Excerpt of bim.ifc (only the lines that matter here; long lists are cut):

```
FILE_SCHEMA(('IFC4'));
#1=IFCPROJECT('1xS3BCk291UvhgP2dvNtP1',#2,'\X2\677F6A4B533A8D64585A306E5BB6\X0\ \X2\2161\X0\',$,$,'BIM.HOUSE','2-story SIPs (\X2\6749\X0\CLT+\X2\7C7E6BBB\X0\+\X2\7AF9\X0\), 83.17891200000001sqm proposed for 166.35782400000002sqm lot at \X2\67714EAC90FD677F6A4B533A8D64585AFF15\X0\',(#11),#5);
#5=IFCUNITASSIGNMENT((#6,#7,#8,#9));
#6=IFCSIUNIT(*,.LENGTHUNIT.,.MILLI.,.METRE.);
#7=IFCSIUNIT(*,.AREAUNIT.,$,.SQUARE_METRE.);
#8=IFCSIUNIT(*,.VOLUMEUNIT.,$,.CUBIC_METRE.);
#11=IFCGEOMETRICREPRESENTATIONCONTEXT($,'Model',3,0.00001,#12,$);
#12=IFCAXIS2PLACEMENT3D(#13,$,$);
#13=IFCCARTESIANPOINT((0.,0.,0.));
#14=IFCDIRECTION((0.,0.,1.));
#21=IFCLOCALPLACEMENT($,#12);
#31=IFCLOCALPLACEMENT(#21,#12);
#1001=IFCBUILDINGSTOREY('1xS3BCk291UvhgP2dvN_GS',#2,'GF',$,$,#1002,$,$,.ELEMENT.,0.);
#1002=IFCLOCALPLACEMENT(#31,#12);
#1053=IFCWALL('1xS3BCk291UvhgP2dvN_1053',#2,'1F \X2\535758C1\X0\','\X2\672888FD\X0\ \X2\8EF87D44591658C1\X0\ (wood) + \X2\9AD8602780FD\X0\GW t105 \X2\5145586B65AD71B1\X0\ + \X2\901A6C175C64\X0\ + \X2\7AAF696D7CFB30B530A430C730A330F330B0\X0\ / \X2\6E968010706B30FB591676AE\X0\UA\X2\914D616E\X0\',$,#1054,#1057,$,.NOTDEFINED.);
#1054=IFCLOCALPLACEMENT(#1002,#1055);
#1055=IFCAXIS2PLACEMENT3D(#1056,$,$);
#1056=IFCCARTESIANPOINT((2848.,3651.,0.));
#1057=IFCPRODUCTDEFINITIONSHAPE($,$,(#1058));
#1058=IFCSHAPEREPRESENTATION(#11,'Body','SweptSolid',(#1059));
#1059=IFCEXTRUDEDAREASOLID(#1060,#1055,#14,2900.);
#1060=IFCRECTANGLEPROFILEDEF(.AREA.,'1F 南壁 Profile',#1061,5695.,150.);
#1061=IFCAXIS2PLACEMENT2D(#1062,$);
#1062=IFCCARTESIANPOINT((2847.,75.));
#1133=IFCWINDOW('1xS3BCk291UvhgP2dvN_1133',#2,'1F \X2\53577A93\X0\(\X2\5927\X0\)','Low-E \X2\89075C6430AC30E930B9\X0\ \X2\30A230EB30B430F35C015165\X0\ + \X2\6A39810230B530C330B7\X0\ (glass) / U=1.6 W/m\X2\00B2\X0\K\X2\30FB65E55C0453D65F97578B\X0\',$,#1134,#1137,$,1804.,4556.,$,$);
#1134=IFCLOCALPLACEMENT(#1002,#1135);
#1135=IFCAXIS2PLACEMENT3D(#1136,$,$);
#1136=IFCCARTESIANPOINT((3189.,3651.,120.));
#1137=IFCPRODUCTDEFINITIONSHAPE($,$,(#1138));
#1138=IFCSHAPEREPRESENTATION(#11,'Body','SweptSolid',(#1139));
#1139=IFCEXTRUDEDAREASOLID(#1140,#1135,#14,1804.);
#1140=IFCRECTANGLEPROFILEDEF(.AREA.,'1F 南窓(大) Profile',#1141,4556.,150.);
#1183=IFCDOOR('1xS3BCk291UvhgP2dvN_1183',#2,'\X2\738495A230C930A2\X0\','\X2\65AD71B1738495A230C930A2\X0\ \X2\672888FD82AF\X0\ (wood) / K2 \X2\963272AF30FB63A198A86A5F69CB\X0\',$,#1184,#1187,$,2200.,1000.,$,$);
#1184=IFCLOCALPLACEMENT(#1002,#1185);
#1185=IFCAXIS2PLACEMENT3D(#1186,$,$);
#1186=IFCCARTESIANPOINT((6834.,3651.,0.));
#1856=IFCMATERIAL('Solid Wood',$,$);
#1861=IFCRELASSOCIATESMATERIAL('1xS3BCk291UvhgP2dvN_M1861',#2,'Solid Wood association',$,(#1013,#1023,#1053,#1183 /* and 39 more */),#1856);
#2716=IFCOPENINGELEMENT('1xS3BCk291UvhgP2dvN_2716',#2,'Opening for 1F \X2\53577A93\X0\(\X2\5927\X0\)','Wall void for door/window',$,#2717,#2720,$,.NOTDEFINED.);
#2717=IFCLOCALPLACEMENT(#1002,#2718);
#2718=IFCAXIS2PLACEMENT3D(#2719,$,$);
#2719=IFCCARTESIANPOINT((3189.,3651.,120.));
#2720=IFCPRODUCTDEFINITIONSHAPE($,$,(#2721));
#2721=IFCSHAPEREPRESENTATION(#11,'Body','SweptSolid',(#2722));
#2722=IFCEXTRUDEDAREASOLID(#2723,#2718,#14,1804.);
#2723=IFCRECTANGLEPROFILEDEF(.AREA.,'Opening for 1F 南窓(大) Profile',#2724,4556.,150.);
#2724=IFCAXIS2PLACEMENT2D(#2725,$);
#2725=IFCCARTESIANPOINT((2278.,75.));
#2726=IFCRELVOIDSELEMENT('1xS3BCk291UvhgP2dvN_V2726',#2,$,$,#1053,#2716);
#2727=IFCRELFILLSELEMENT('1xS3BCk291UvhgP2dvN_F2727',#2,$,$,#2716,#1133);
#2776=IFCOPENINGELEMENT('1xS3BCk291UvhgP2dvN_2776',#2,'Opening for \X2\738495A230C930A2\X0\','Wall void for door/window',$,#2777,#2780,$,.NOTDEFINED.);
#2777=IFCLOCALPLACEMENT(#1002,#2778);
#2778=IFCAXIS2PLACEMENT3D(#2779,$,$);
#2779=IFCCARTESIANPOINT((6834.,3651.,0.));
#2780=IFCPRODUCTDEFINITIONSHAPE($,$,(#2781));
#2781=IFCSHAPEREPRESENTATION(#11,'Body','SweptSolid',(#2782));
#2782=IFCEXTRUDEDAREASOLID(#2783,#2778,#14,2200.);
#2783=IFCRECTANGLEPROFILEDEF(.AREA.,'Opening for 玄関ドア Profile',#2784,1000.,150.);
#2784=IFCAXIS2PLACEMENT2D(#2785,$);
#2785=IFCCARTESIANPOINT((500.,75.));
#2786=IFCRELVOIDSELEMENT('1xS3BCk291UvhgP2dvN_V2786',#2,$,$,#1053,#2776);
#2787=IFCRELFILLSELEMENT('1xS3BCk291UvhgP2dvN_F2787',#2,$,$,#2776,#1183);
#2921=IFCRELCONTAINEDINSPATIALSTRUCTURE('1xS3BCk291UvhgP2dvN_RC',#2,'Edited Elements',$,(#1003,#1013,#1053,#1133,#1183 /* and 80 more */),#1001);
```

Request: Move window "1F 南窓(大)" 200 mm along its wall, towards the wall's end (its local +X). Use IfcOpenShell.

```python
import ifcopenshell
import ifcopenshell.api.geometry
import ifcopenshell.util.placement
import ifcopenshell.util.unit

model = ifcopenshell.open("bim.ifc")
unit_scale = ifcopenshell.util.unit.calculate_unit_scale(model)

window = model.by_id(1133)
opening = window.FillsVoids[0].RelatingOpeningElement
wall = opening.VoidsElements[0].RelatingBuildingElement

wall_matrix = ifcopenshell.util.placement.get_local_placement(wall.ObjectPlacement)
shift = wall_matrix[:3, 0] * 0.2 / unit_scale
before = ifcopenshell.util.placement.get_local_placement(window.ObjectPlacement)[:3, 3].copy()

# The window is not placed relative to its opening, so move both.
for product in (opening, window):
    matrix = ifcopenshell.util.placement.get_local_placement(product.ObjectPlacement)
    matrix[:3, 3] += shift
    ifcopenshell.api.geometry.edit_object_placement(model, product=product, matrix=matrix, is_si=False)

after = ifcopenshell.util.placement.get_local_placement(window.ObjectPlacement)[:3, 3]
print("window moved by", (after - before).round(3) + 0.0)

model.write("bim_rev.ifc")
```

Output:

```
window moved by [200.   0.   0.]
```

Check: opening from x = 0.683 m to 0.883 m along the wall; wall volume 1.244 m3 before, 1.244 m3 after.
